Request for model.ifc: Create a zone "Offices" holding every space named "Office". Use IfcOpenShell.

First a look at what the model holds.

```python
import ifcopenshell

model = ifcopenshell.open("model.ifc")
print(model.schema)
seen = {}
for space in model.by_type("IfcSpace"):
    seen[space.LongName] = seen.get(space.LongName, 0) + 1
for name, count in sorted(seen.items(), key=str):
    print(count, "x", name)
print("zones:", [z.Name for z in model.by_type("IfcZone")][:20])
```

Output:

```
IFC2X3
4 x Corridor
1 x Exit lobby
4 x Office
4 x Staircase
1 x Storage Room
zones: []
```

```python
import ifcopenshell
import ifcopenshell.api.group
import ifcopenshell.api.root

model = ifcopenshell.open("model.ifc")

names = {"Office"}
spaces = [s for s in model.by_type("IfcSpace") if s.LongName in names]

zone = ifcopenshell.api.root.create_entity(model, ifc_class="IfcZone", name="Offices")
ifcopenshell.api.group.assign_group(model, products=spaces, group=zone)
print(len(spaces), "spaces in", zone.Name)

model.write("model_v2.ifc")
```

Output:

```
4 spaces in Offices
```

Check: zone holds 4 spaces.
